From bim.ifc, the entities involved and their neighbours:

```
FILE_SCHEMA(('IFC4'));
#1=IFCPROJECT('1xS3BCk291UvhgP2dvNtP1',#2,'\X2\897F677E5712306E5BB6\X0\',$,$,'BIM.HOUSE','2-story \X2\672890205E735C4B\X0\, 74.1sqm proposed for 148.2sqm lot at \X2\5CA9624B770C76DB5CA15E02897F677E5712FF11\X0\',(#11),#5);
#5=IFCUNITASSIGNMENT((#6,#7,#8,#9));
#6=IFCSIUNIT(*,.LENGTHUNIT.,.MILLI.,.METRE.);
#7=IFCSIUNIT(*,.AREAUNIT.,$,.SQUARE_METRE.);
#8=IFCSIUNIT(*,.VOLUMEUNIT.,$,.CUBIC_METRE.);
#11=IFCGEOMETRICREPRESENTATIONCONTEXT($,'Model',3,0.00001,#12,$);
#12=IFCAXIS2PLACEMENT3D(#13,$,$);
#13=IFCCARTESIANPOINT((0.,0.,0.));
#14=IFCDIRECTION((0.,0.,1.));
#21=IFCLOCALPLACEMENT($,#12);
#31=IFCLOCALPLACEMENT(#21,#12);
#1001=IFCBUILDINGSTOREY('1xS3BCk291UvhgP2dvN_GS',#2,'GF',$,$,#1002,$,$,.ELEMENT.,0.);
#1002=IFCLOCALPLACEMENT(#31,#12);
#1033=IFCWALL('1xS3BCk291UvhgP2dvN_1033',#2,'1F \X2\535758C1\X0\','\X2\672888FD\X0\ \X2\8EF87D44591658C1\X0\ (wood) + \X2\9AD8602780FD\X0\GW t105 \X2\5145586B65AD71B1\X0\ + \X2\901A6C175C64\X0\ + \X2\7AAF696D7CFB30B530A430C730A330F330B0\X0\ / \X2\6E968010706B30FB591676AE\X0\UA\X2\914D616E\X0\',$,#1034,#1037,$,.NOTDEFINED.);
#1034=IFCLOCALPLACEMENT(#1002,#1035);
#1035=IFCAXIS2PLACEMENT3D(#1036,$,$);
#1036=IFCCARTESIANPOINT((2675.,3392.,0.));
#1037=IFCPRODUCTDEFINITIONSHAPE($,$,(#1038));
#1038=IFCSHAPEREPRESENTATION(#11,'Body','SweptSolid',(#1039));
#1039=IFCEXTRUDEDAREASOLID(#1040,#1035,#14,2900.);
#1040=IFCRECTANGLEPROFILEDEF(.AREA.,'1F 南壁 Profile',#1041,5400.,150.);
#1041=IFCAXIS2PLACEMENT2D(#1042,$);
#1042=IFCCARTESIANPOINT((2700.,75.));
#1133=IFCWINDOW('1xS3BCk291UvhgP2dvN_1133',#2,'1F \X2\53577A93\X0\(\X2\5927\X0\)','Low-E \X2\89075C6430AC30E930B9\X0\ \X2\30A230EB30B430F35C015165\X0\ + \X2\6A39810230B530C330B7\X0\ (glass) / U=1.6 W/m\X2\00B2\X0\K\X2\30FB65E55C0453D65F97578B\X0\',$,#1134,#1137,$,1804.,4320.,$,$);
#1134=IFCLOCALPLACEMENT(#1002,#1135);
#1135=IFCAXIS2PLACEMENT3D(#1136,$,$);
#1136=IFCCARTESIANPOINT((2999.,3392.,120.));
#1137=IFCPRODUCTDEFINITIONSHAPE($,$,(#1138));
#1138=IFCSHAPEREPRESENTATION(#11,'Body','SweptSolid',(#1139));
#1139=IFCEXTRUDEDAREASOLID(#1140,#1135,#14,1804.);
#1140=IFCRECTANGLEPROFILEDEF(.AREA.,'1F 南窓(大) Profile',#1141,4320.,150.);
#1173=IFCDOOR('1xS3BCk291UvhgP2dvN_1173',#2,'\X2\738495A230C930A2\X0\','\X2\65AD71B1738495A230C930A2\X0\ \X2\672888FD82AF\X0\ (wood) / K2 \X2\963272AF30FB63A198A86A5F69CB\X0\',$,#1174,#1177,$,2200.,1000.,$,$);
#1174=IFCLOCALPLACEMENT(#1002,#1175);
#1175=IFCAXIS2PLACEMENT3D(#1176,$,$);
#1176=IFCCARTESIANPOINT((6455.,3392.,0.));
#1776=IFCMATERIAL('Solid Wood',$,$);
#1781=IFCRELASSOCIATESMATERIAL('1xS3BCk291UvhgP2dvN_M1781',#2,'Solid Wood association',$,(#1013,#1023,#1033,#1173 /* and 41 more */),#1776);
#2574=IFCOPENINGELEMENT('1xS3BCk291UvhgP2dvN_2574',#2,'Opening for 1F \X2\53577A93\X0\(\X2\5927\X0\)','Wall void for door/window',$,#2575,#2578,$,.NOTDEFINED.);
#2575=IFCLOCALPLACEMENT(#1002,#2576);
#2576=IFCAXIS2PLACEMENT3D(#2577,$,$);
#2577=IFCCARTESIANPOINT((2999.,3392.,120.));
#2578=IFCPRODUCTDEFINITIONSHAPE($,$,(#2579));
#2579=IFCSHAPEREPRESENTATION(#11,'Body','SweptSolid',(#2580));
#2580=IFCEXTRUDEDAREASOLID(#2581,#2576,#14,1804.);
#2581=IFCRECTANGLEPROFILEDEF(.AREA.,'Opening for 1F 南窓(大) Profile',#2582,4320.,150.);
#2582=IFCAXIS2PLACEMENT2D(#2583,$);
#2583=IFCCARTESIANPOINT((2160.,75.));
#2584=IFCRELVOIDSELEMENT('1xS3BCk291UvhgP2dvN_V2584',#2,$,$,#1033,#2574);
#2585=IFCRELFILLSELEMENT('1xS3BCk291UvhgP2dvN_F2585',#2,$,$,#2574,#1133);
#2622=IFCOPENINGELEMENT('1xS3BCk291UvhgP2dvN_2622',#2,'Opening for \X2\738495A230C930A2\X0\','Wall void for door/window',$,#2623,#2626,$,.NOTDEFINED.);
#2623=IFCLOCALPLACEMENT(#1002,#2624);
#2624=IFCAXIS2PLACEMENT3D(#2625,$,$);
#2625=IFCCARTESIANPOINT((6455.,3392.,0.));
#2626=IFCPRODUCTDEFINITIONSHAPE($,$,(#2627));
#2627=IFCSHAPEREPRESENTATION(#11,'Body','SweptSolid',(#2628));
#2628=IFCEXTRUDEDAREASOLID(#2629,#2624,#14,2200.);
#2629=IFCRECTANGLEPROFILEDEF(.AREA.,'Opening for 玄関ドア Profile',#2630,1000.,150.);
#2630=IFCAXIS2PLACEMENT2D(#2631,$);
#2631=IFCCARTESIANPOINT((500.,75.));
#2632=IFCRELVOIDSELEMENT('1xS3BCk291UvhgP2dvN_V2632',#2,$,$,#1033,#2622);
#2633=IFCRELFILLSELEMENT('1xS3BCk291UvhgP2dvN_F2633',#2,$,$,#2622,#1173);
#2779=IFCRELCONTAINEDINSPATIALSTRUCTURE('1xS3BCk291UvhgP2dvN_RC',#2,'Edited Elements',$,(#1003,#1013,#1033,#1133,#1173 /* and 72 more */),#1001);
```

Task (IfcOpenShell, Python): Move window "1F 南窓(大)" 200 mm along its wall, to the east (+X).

```python
import ifcopenshell
import ifcopenshell.api.geometry
import ifcopenshell.util.placement
import ifcopenshell.util.unit

model = ifcopenshell.open("bim.ifc")
unit_scale = ifcopenshell.util.unit.calculate_unit_scale(model)

window = model.by_id(1133)
opening = window.FillsVoids[0].RelatingOpeningElement
wall = opening.VoidsElements[0].RelatingBuildingElement

wall_matrix = ifcopenshell.util.placement.get_local_placement(wall.ObjectPlacement)
shift = wall_matrix[:3, 0] * 0.2 / unit_scale
before = ifcopenshell.util.placement.get_local_placement(window.ObjectPlacement)[:3, 3].copy()

# The window is not placed relative to its opening, so move both.
for product in (opening, window):
    matrix = ifcopenshell.util.placement.get_local_placement(product.ObjectPlacement)
    matrix[:3, 3] += shift
    ifcopenshell.api.geometry.edit_object_placement(model, product=product, matrix=matrix, is_si=False)

after = ifcopenshell.util.placement.get_local_placement(window.ObjectPlacement)[:3, 3]
print("window moved by", (after - before).round(3) + 0.0)

model.write("bim_updated.ifc")
```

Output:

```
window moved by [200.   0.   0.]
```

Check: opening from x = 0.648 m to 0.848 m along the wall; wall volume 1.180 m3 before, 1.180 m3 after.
